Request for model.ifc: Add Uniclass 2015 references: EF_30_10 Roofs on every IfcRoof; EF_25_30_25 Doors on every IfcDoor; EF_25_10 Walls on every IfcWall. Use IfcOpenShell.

First a look at what the model holds.

```python
import ifcopenshell

model = ifcopenshell.open("model.ifc")
print(model.schema)
print("classifications:", [c.Name for c in model.by_type("IfcClassification")])
for ifc_class in ("IfcDoor", "IfcRoof", "IfcStair", "IfcWall", "IfcWindow"):
    print(ifc_class, len(model.by_type(ifc_class)))
```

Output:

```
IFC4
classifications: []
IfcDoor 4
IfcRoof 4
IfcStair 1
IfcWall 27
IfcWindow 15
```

```python
import ifcopenshell
import ifcopenshell.api.classification

model = ifcopenshell.open("model.ifc")

system = ifcopenshell.api.classification.add_classification(model, classification="Uniclass 2015")

codes = {
    "IfcRoof": ("EF_30_10", "Roofs"),
    "IfcDoor": ("EF_25_30_25", "Doors"),
    "IfcWall": ("EF_25_10", "Walls"),
}
for ifc_class, (code, name) in codes.items():
    products = model.by_type(ifc_class)
    ifcopenshell.api.classification.add_reference(
        model, products=products, classification=system, identification=code, name=name
    )
    print(code, len(products))

model.write("model_edited.ifc")
```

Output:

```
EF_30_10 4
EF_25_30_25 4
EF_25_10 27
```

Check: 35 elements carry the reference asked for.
